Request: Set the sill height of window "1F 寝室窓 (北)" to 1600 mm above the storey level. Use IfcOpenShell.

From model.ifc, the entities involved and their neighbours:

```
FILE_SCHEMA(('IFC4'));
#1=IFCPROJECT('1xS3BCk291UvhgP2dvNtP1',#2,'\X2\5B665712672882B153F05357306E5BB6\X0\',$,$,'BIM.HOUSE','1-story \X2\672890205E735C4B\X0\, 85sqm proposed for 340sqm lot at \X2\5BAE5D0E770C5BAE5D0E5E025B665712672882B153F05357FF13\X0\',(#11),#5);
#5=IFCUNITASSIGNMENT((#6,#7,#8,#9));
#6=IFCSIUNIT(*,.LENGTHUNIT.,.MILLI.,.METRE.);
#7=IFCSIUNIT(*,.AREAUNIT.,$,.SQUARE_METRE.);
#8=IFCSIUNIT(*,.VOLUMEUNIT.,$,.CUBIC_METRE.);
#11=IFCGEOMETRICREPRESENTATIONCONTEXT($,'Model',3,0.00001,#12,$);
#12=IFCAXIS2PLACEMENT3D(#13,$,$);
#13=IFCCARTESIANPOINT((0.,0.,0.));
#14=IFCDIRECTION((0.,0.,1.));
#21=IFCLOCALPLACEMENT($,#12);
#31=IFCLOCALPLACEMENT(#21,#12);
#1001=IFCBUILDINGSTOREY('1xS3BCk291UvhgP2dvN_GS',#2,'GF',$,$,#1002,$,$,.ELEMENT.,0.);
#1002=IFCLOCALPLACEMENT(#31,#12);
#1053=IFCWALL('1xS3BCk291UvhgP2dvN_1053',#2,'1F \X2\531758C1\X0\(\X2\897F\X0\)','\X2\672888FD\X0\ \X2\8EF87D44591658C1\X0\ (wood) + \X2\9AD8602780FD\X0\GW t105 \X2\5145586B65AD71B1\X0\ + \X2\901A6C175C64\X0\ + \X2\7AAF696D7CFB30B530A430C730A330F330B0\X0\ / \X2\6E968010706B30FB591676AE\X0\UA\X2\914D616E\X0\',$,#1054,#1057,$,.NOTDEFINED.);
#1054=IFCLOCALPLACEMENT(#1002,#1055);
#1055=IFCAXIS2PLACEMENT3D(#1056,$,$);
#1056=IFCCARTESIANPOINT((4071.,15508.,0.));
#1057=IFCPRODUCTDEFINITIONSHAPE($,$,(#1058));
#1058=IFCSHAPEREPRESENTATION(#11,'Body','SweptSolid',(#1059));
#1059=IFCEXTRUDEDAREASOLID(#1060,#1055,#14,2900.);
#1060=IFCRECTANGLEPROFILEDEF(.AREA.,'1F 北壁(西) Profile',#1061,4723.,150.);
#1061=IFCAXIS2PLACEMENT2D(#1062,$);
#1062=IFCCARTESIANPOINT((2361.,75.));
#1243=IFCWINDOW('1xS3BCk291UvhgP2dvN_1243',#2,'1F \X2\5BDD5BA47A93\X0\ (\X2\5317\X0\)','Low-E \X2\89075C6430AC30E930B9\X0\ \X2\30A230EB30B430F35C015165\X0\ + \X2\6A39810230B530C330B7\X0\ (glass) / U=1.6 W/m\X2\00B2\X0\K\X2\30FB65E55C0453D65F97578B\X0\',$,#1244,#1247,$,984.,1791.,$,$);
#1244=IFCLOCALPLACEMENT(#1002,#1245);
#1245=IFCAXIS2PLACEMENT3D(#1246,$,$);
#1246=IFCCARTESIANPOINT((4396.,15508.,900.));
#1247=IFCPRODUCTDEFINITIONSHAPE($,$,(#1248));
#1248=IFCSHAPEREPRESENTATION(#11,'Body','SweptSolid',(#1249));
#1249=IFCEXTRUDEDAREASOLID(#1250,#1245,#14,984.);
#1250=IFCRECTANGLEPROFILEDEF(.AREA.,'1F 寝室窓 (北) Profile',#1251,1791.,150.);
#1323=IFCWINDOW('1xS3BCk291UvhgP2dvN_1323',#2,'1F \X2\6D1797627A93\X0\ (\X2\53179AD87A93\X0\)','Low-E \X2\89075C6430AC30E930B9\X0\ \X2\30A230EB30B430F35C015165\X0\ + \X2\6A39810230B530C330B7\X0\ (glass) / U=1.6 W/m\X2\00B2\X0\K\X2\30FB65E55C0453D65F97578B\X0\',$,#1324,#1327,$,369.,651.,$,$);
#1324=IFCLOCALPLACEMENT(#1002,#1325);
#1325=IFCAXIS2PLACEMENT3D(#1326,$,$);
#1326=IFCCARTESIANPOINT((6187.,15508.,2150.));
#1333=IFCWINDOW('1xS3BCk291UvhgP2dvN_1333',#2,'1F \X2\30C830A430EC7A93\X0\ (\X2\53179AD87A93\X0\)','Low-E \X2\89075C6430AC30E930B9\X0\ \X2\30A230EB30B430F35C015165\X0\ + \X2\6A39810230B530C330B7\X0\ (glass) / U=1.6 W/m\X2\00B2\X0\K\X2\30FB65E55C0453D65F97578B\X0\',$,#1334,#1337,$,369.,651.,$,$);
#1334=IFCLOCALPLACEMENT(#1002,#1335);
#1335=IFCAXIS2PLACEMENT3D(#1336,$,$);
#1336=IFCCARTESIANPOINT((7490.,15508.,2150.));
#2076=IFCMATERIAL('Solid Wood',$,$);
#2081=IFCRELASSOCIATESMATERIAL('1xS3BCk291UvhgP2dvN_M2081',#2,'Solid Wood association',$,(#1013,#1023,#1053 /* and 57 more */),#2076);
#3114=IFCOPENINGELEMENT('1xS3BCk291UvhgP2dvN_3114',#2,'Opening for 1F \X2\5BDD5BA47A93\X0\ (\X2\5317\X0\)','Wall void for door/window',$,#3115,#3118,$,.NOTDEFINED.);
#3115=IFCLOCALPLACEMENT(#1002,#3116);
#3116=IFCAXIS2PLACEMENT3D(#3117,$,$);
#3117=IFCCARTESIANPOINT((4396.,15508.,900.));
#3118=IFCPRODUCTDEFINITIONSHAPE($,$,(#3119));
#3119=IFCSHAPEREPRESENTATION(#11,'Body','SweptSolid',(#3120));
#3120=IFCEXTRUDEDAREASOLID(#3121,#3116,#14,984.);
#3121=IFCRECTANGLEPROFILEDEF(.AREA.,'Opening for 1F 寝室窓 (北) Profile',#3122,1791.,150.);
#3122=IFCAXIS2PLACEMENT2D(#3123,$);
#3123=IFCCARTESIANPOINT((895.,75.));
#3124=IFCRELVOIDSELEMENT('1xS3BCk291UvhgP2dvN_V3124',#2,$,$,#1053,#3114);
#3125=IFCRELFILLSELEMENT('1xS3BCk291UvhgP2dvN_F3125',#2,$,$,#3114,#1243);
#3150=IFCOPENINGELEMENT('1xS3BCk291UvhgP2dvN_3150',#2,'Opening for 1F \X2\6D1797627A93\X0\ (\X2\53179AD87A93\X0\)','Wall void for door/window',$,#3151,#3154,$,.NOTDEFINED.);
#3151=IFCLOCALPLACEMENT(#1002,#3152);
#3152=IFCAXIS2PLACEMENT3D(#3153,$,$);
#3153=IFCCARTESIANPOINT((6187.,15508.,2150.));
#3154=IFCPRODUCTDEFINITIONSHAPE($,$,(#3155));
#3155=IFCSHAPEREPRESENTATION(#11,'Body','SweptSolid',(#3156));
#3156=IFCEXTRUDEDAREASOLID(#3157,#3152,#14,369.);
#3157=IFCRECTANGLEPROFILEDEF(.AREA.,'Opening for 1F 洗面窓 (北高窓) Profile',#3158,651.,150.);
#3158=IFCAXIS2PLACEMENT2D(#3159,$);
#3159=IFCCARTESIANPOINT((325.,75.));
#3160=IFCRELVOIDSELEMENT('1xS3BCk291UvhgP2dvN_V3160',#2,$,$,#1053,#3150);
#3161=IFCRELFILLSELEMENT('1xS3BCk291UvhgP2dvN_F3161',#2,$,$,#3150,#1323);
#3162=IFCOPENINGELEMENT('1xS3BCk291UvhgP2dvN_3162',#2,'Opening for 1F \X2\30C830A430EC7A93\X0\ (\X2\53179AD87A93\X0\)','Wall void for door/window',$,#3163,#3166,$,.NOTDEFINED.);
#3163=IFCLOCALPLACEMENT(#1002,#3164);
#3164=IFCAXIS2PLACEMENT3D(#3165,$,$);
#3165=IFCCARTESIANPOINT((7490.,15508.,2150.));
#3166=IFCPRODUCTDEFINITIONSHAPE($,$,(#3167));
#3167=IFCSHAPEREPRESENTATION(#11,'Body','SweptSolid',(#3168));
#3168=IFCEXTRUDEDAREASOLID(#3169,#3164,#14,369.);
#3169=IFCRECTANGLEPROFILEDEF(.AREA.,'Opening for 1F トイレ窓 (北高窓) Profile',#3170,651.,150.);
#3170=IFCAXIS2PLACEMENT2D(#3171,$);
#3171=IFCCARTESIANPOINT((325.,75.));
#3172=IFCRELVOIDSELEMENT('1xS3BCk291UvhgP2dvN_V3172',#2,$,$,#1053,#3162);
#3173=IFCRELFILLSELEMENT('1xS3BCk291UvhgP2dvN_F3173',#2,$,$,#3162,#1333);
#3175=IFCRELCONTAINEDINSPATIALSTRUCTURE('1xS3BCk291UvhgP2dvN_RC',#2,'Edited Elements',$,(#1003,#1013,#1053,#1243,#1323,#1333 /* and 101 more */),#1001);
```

```python
import numpy as np
import ifcopenshell
import ifcopenshell.api.geometry
import ifcopenshell.geom
import ifcopenshell.util.element
import ifcopenshell.util.placement
import ifcopenshell.util.shape
import ifcopenshell.util.unit

model = ifcopenshell.open("model.ifc")
unit_scale = ifcopenshell.util.unit.calculate_unit_scale(model)

window = model.by_guid("1xS3BCk291UvhgP2dvN_1243")
opening = window.FillsVoids[0].RelatingOpeningElement
storey = ifcopenshell.util.element.get_container(window, ifc_class="IfcBuildingStorey")
level = ifcopenshell.util.placement.get_local_placement(storey.ObjectPlacement)[2, 3]

# The opening's origin need not be at the sill, so measure its lowest point.
shape = ifcopenshell.geom.create_shape(ifcopenshell.geom.settings(), opening)
bottom = ifcopenshell.util.shape.get_shape_bottom_elevation(shape, shape.geometry) / unit_scale
dz = level + 1.6 / unit_scale - bottom

shift = np.array([0.0, 0.0, dz])
# The window is not placed relative to its opening, so move both.
for product in (opening, window):
    matrix = ifcopenshell.util.placement.get_local_placement(product.ObjectPlacement)
    matrix[:3, 3] += shift
    ifcopenshell.api.geometry.edit_object_placement(model, product=product, matrix=matrix, is_si=False)

print(f"moved by {dz * unit_scale:+.3f} m")

model.write("model_v2.ifc")
```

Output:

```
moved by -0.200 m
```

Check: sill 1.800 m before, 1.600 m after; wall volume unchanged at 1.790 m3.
